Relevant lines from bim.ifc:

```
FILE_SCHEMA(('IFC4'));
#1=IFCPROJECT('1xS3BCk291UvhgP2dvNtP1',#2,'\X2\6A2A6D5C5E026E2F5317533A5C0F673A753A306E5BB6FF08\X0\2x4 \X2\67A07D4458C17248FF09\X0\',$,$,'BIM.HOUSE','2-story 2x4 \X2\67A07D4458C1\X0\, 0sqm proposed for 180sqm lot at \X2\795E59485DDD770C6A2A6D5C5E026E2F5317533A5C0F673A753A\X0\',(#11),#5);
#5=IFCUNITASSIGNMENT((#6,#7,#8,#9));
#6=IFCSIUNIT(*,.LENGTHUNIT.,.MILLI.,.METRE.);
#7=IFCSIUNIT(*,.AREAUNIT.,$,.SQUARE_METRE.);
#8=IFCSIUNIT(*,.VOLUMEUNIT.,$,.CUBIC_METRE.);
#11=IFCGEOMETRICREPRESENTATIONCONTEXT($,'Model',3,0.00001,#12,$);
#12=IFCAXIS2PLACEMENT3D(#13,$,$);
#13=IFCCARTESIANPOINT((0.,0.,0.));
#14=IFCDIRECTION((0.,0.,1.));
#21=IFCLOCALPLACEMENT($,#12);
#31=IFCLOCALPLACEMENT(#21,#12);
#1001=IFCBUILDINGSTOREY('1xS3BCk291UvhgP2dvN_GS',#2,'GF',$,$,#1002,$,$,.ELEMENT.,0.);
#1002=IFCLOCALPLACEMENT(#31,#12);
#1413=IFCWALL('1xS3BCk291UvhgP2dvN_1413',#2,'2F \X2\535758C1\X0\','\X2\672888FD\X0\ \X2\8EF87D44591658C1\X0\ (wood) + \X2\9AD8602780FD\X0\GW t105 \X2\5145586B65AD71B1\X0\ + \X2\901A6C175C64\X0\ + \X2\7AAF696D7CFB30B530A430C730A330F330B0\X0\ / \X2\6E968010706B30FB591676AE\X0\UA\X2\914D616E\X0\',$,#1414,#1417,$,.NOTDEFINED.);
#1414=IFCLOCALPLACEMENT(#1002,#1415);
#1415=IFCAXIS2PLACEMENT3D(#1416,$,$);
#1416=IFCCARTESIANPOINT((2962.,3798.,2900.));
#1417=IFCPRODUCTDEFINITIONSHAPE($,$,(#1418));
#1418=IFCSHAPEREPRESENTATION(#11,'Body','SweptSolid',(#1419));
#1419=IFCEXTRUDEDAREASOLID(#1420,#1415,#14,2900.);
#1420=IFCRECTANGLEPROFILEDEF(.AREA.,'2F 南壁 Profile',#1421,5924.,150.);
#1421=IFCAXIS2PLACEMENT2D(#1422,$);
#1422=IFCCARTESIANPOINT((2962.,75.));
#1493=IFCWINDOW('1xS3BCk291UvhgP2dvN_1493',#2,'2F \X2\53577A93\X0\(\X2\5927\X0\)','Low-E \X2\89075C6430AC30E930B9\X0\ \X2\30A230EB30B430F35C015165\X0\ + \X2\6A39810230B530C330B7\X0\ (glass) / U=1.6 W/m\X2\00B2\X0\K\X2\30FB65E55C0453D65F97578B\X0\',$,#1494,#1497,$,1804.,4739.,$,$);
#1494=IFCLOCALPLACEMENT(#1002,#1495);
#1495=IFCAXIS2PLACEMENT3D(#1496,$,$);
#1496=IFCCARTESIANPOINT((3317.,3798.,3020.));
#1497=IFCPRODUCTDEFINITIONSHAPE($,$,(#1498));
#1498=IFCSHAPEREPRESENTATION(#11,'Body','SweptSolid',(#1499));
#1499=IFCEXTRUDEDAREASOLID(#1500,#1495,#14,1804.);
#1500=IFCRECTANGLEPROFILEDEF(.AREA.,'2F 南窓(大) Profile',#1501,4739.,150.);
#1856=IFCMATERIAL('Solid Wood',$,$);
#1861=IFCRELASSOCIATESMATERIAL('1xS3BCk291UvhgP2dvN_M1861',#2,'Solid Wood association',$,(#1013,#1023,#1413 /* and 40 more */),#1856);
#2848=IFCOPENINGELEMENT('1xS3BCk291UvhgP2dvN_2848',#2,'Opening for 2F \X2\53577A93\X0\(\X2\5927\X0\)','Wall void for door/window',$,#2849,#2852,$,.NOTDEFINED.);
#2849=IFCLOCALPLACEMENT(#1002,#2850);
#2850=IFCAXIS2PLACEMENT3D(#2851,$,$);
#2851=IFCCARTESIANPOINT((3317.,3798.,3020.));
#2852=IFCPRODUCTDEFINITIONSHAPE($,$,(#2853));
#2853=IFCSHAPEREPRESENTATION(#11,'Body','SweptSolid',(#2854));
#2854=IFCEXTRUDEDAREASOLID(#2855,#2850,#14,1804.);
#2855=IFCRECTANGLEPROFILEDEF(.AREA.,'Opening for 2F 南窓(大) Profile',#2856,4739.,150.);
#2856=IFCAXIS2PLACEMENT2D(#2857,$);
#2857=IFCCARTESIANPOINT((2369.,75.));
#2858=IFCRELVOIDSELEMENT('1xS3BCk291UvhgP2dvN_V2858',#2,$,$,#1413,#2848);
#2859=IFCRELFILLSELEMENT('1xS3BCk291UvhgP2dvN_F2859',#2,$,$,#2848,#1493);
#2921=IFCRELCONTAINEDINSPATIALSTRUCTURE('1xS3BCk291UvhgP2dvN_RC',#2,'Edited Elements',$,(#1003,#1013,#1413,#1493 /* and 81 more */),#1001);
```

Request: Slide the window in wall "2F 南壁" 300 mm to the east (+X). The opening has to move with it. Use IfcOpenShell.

```python
import ifcopenshell
import ifcopenshell.api.geometry
import ifcopenshell.util.placement

model = ifcopenshell.open("bim.ifc")

window = model.by_guid("1xS3BCk291UvhgP2dvN_1493")
opening = window.FillsVoids[0].RelatingOpeningElement
wall = opening.VoidsElements[0].RelatingBuildingElement

wall_matrix = ifcopenshell.util.placement.get_local_placement(wall.ObjectPlacement)
shift = wall_matrix[:3, 0] * 300.0
before = ifcopenshell.util.placement.get_local_placement(window.ObjectPlacement)[:3, 3].copy()

# The window is not placed relative to its opening, so move both.
for product in (opening, window):
    matrix = ifcopenshell.util.placement.get_local_placement(product.ObjectPlacement)
    matrix[:3, 3] += shift
    ifcopenshell.api.geometry.edit_object_placement(model, product=product, matrix=matrix, is_si=False)

after = ifcopenshell.util.placement.get_local_placement(window.ObjectPlacement)[:3, 3]
print("window moved by", (after - before).round(3) + 0.0)

model.write("bim_v2.ifc")
```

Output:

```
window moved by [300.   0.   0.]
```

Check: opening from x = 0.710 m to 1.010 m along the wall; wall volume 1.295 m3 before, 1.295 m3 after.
